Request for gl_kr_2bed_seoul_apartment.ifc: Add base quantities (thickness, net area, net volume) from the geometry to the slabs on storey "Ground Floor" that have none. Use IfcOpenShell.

First a look at what the model holds.

```python
import ifcopenshell
import ifcopenshell.util.element
import ifcopenshell.util.unit

model = ifcopenshell.open("gl_kr_2bed_seoul_apartment.ifc")
print(model.schema)
for unit_type in ("LENGTHUNIT", "AREAUNIT", "VOLUMEUNIT"):
    print(unit_type, ifcopenshell.util.unit.calculate_unit_scale(model, unit_type))
storey = next(s for s in model.by_type("IfcBuildingStorey") if s.Name == "Ground Floor")
slabs = [e for e in ifcopenshell.util.element.get_decomposition(storey) if e.is_a("IfcSlab")]
for e in sorted(slabs, key=lambda e: e.id()):
    print(e.id(), e.is_a(), e.Name, list(ifcopenshell.util.element.get_psets(e, qtos_only=True)), sep=" | ")
```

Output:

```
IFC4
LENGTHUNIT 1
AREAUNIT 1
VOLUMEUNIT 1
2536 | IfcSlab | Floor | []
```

```python
import ifcopenshell
import ifcopenshell.api.pset
import ifcopenshell.geom
import ifcopenshell.util.element
import ifcopenshell.util.shape
import ifcopenshell.util.unit

model = ifcopenshell.open("gl_kr_2bed_seoul_apartment.ifc")
unit_scale = ifcopenshell.util.unit.calculate_unit_scale(model)
area_scale = ifcopenshell.util.unit.calculate_unit_scale(model, "AREAUNIT")
volume_scale = ifcopenshell.util.unit.calculate_unit_scale(model, "VOLUMEUNIT")
settings = ifcopenshell.geom.settings()

storey = next(s for s in model.by_type("IfcBuildingStorey") if s.Name == "Ground Floor")
slabs = [e for e in ifcopenshell.util.element.get_decomposition(storey) if e.is_a("IfcSlab")]

for e in sorted(slabs, key=lambda e: e.id()):
    if ifcopenshell.util.element.get_psets(e, qtos_only=True, should_inherit=False):
        continue
    # Geometry comes back in metres, in the element's own axes.
    shape = ifcopenshell.geom.create_shape(settings, e)
    values = {
        "Width": ifcopenshell.util.shape.get_z(shape.geometry) / unit_scale,
        "NetArea": ifcopenshell.util.shape.get_footprint_area(shape.geometry) / area_scale,
        "NetVolume": ifcopenshell.util.shape.get_volume(shape.geometry) / volume_scale,
    }
    qto = ifcopenshell.api.pset.add_qto(model, product=e, name="Qto_SlabBaseQuantities")
    ifcopenshell.api.pset.edit_qto(model, qto=qto, properties=values)
    print(e.id(), {k: round(v, 3) for k, v in values.items()})

model.write("gl_kr_2bed_seoul_apartment-out.ifc")
```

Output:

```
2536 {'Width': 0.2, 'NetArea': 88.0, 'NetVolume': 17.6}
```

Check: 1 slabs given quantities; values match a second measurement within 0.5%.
